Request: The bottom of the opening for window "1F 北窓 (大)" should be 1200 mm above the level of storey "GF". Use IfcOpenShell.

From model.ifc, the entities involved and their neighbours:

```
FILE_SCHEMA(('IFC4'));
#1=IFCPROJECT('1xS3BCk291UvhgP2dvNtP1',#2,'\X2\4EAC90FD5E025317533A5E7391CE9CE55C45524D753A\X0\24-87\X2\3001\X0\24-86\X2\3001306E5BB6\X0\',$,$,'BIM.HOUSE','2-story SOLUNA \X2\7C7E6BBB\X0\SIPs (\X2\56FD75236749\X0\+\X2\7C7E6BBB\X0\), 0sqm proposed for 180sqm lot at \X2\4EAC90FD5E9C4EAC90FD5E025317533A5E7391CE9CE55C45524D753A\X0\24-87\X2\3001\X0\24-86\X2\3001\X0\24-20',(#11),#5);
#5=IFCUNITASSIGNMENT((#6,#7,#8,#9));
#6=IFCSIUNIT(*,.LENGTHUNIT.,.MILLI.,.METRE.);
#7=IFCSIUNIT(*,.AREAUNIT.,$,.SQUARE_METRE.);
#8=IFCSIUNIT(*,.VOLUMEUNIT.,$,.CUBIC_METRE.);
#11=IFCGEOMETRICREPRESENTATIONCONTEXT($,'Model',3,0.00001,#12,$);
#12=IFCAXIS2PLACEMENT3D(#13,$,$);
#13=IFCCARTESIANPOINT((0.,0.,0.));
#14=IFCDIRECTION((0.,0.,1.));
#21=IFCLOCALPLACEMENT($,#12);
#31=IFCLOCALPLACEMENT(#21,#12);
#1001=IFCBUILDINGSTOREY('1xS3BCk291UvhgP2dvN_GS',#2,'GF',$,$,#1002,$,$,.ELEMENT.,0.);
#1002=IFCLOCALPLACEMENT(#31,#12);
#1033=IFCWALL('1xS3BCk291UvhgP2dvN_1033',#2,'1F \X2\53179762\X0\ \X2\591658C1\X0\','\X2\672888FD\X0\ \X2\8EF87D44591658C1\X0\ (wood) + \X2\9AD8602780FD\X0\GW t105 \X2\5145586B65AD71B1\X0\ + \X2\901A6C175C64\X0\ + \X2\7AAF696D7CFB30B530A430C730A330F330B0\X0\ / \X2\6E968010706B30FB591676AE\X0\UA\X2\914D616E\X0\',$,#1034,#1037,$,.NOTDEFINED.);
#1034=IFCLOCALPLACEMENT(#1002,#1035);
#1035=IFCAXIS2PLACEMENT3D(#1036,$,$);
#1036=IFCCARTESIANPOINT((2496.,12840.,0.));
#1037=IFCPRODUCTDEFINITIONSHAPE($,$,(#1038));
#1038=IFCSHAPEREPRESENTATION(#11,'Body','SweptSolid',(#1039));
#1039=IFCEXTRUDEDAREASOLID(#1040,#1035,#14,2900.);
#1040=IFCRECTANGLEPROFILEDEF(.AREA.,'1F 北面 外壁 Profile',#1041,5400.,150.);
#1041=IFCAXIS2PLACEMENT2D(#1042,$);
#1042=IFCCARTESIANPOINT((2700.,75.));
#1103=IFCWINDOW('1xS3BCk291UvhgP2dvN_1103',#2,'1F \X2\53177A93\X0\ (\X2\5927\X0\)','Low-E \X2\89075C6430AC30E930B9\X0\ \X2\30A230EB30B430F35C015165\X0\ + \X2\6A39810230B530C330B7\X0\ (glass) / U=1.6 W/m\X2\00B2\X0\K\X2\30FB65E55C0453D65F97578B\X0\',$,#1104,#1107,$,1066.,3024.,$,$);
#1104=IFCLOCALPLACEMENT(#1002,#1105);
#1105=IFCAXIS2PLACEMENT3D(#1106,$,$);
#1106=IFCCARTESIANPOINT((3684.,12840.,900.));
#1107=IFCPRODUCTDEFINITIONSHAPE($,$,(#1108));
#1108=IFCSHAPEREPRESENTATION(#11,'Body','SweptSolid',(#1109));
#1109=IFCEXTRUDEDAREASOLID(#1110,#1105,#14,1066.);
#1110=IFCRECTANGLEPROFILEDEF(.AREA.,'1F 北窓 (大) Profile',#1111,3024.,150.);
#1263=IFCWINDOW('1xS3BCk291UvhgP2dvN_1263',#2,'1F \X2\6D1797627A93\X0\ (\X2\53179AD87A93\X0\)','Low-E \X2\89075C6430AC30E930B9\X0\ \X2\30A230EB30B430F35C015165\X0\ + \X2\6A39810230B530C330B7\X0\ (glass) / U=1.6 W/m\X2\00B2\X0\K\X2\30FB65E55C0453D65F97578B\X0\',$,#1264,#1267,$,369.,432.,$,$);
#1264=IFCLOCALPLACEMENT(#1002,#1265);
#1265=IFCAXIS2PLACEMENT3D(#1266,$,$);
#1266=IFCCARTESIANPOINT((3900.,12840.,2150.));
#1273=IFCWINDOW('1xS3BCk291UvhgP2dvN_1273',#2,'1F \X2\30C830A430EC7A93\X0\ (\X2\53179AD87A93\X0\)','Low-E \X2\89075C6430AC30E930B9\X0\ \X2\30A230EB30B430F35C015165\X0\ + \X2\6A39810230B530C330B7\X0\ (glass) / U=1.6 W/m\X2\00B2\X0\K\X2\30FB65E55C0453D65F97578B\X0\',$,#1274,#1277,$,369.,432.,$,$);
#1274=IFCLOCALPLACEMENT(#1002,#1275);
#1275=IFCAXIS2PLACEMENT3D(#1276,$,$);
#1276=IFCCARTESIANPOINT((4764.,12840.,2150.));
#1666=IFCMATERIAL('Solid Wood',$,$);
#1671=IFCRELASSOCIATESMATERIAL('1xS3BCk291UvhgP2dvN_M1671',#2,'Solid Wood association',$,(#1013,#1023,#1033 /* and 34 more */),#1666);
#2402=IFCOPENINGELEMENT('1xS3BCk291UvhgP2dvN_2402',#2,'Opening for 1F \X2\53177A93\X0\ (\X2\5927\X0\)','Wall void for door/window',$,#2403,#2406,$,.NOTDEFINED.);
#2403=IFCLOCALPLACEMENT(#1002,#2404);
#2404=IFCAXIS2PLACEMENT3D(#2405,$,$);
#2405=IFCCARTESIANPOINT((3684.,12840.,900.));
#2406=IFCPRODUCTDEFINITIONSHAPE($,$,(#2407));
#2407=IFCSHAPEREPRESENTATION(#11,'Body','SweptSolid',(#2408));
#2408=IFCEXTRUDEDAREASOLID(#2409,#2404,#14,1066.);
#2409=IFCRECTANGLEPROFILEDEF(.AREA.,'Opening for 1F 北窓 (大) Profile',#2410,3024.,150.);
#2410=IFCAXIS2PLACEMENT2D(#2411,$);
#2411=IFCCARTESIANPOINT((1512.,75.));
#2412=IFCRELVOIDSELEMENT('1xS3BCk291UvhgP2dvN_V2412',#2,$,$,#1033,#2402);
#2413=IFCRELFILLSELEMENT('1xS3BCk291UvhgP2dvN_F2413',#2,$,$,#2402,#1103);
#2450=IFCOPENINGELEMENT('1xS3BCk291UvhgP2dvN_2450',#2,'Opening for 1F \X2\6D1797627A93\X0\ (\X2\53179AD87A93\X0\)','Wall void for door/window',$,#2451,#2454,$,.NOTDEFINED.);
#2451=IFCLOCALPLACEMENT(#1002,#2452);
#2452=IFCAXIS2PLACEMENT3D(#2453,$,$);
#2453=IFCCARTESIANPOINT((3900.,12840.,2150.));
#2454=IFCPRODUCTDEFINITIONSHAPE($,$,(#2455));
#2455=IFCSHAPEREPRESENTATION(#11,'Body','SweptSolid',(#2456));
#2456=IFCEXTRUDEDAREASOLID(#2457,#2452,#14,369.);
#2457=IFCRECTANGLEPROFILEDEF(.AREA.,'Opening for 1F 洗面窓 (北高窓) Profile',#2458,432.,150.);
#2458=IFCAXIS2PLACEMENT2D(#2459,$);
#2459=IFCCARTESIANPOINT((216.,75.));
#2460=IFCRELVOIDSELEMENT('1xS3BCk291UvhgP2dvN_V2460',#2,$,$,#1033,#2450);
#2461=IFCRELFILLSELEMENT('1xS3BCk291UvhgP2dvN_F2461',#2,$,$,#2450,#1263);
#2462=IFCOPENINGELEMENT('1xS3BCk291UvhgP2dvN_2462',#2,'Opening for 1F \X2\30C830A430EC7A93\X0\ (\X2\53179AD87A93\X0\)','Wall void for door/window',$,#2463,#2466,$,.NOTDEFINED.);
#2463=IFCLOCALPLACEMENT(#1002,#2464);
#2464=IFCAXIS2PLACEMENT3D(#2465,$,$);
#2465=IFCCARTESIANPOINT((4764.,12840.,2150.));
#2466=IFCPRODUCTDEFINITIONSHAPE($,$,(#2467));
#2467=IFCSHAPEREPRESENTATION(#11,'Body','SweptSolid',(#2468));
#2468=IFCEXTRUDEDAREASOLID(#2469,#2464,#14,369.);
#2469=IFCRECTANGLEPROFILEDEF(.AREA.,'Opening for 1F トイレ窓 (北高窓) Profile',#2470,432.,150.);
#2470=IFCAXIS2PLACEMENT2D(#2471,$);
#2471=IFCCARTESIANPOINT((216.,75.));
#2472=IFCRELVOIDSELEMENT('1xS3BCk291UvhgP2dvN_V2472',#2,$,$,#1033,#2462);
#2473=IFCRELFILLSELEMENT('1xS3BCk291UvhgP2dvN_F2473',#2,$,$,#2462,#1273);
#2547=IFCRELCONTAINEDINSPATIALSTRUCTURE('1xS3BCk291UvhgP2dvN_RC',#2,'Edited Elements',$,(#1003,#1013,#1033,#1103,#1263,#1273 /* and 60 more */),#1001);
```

```python
import numpy as np
import ifcopenshell
import ifcopenshell.api.geometry
import ifcopenshell.geom
import ifcopenshell.util.element
import ifcopenshell.util.placement
import ifcopenshell.util.shape
import ifcopenshell.util.unit

model = ifcopenshell.open("model.ifc")
unit_scale = ifcopenshell.util.unit.calculate_unit_scale(model)

window = model.by_id(1103)
opening = window.FillsVoids[0].RelatingOpeningElement
storey = ifcopenshell.util.element.get_container(window, ifc_class="IfcBuildingStorey")
level = ifcopenshell.util.placement.get_local_placement(storey.ObjectPlacement)[2, 3]

# The opening's origin need not be at the sill, so measure its lowest point.
shape = ifcopenshell.geom.create_shape(ifcopenshell.geom.settings(), opening)
bottom = ifcopenshell.util.shape.get_shape_bottom_elevation(shape, shape.geometry) / unit_scale
dz = level + 1.2 / unit_scale - bottom

shift = np.array([0.0, 0.0, dz])
# The window is not placed relative to its opening, so move both.
for product in (opening, window):
    matrix = ifcopenshell.util.placement.get_local_placement(product.ObjectPlacement)
    matrix[:3, 3] += shift
    ifcopenshell.api.geometry.edit_object_placement(model, product=product, matrix=matrix, is_si=False)

print(f"moved by {dz * unit_scale:+.3f} m")

model.write("model-out.ifc")
```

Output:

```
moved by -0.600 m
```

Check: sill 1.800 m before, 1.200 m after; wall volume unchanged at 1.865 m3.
